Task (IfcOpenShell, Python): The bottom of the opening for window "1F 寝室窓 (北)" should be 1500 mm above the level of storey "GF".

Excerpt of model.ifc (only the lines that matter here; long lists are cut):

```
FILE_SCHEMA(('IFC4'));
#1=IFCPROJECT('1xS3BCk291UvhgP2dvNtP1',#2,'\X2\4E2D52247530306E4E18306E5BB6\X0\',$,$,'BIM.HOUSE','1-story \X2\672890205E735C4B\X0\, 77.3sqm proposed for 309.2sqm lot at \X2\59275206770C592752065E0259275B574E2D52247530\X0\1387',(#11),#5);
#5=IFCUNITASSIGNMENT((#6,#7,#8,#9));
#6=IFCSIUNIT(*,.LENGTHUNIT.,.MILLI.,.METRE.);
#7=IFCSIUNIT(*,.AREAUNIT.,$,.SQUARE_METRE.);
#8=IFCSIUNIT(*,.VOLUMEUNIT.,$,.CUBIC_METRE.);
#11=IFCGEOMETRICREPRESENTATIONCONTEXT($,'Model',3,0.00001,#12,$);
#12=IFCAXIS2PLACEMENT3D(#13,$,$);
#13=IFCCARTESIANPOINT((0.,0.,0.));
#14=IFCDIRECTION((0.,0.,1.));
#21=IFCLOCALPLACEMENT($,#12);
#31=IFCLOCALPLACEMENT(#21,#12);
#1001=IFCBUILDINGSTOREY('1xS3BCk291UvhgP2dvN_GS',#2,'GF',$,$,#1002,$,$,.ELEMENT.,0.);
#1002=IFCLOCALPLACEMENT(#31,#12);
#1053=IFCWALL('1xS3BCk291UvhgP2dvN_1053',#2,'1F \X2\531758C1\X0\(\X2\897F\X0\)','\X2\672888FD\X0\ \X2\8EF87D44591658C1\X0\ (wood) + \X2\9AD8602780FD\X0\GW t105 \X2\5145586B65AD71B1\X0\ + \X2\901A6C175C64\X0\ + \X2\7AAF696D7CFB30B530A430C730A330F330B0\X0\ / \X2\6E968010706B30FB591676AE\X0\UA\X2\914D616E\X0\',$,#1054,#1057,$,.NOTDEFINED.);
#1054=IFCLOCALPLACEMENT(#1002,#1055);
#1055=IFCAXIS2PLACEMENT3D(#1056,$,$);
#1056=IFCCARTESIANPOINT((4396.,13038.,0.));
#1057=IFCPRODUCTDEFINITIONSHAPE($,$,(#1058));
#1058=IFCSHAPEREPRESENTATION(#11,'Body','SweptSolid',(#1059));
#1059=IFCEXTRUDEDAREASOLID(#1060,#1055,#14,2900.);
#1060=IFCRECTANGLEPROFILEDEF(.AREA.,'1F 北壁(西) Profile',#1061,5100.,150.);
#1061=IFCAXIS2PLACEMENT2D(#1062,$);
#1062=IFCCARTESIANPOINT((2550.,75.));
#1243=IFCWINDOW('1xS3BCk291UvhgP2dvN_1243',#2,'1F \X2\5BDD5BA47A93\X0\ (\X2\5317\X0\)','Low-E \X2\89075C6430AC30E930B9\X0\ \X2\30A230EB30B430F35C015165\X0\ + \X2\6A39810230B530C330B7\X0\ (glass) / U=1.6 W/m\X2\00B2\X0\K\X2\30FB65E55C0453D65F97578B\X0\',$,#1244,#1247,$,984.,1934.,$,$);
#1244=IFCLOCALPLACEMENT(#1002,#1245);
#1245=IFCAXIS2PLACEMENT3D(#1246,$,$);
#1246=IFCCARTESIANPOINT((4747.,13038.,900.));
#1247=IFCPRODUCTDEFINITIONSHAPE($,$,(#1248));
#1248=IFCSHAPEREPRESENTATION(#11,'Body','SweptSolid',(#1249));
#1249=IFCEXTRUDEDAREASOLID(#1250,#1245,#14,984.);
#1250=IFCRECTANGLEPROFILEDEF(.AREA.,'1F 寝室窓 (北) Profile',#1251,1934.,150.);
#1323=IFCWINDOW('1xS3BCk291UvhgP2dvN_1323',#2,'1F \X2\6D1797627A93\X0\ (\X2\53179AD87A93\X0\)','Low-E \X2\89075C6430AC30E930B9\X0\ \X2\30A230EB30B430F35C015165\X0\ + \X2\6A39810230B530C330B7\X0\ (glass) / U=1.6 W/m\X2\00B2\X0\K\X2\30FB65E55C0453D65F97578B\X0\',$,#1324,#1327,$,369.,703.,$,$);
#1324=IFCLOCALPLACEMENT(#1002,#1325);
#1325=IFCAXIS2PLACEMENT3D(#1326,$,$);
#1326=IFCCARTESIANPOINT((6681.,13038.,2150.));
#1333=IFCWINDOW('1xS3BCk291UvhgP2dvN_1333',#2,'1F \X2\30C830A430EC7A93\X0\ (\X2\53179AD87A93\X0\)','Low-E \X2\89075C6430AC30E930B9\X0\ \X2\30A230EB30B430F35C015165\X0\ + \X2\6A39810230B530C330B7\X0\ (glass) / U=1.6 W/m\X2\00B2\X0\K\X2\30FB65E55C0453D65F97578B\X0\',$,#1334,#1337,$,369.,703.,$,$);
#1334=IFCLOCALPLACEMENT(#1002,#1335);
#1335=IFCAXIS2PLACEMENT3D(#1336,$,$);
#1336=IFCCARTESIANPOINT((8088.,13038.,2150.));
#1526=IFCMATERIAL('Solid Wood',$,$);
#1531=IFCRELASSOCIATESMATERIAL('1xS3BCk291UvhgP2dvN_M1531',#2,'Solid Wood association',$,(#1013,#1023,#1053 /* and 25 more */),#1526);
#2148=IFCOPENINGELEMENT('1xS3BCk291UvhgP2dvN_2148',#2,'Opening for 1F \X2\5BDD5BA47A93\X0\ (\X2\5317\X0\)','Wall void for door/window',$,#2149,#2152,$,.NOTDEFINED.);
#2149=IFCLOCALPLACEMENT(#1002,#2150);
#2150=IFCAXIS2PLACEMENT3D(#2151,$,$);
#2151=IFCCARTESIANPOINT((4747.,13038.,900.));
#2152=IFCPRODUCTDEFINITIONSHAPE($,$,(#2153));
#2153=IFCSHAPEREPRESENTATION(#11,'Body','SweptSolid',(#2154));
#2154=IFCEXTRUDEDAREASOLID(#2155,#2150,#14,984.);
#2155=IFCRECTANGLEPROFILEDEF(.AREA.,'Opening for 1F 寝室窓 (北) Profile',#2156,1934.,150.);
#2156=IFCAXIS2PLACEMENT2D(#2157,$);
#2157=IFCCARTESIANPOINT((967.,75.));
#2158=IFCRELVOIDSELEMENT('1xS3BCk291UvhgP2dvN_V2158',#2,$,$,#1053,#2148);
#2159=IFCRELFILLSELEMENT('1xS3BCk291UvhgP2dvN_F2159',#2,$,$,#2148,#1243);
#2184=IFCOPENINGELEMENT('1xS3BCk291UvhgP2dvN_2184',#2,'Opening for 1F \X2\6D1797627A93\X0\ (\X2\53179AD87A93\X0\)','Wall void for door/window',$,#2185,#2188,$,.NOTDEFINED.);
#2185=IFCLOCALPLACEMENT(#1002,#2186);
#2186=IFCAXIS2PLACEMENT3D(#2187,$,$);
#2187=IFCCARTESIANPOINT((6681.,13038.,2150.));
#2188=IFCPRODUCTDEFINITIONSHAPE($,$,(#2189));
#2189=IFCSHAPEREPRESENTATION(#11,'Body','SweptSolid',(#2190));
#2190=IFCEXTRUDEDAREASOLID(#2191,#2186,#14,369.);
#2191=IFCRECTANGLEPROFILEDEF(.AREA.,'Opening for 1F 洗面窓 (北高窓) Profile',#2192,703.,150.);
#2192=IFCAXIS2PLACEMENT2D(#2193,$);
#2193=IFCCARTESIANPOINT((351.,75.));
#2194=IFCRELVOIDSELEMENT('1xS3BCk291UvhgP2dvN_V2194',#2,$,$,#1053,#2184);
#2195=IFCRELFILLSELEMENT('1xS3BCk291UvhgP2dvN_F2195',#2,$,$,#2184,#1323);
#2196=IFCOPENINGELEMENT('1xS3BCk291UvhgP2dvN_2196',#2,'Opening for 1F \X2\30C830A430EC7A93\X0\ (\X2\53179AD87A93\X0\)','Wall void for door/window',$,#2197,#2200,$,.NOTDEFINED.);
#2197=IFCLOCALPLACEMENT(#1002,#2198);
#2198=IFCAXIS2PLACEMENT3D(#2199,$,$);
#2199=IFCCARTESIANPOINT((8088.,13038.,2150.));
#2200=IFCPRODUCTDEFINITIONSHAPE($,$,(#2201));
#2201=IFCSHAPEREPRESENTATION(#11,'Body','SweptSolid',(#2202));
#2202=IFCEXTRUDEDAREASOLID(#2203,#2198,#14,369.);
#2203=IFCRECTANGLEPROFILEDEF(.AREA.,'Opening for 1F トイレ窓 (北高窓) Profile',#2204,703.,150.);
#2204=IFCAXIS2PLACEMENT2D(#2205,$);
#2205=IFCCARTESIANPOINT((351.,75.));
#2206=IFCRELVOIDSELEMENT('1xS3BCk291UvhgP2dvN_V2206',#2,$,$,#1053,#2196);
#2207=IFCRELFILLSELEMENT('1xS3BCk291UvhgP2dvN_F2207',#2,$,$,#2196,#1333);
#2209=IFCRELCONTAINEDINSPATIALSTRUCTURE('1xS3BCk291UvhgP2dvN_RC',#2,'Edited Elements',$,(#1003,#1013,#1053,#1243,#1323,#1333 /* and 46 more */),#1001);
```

```python
import numpy as np
import ifcopenshell
import ifcopenshell.api.geometry
import ifcopenshell.geom
import ifcopenshell.util.element
import ifcopenshell.util.placement
import ifcopenshell.util.shape
import ifcopenshell.util.unit

model = ifcopenshell.open("model.ifc")
unit_scale = ifcopenshell.util.unit.calculate_unit_scale(model)

window = model.by_guid("1xS3BCk291UvhgP2dvN_1243")
opening = window.FillsVoids[0].RelatingOpeningElement
storey = ifcopenshell.util.element.get_container(window, ifc_class="IfcBuildingStorey")
level = ifcopenshell.util.placement.get_local_placement(storey.ObjectPlacement)[2, 3]

# The opening's origin need not be at the sill, so measure its lowest point.
shape = ifcopenshell.geom.create_shape(ifcopenshell.geom.settings(), opening)
bottom = ifcopenshell.util.shape.get_shape_bottom_elevation(shape, shape.geometry) / unit_scale
dz = level + 1.5 / unit_scale - bottom

shift = np.array([0.0, 0.0, dz])
# The window is not placed relative to its opening, so move both.
for product in (opening, window):
    matrix = ifcopenshell.util.placement.get_local_placement(product.ObjectPlacement)
    matrix[:3, 3] += shift
    ifcopenshell.api.geometry.edit_object_placement(model, product=product, matrix=matrix, is_si=False)

print(f"moved by {dz * unit_scale:+.3f} m")

model.write("model_updated.ifc")
```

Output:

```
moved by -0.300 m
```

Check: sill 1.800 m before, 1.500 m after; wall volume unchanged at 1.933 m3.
